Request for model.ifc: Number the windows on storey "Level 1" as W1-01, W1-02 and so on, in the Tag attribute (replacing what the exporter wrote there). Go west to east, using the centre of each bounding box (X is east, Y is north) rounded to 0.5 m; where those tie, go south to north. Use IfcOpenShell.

First a look at what the model holds.

```python
import ifcopenshell
import ifcopenshell.util.element
import ifcopenshell.util.placement

model = ifcopenshell.open("model.ifc")
print(model.schema)
storey = next(s for s in model.by_type("IfcBuildingStorey") if s.Name == "Level 1")
windows = [e for e in ifcopenshell.util.element.get_decomposition(storey) if e.is_a("IfcWindow")]
for e in sorted(windows, key=lambda e: e.id()):
    origin = ifcopenshell.util.placement.get_local_placement(e.ObjectPlacement)[:3, 3]
    print(e.id(), e.Tag, e.Name, origin.round(2) + 0.0, sep=" | ")
```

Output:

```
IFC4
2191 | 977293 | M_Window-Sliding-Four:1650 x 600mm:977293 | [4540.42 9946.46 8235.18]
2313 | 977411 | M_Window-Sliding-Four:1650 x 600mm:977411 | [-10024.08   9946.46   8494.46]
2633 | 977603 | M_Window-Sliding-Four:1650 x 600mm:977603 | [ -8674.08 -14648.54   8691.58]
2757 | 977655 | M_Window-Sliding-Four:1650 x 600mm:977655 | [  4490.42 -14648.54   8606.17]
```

```python
import ifcopenshell
import ifcopenshell.geom
import ifcopenshell.util.element
import ifcopenshell.util.shape

model = ifcopenshell.open("model.ifc")
settings = ifcopenshell.geom.settings()
settings.set("use-world-coords", True)


def centre(element):
    shape = ifcopenshell.geom.create_shape(settings, element)
    return ifcopenshell.util.shape.get_bbox_centroid(shape.geometry)


storey = next(s for s in model.by_type("IfcBuildingStorey") if s.Name == "Level 1")
windows = [e for e in ifcopenshell.util.element.get_decomposition(storey) if e.is_a("IfcWindow")]

# Insertion points can sit at a corner or the storey origin, so sort by the geometry (in metres).
centres = {e: centre(e) for e in windows}
windows.sort(key=lambda e: (round(centres[e][0] / 0.5), centres[e][1]))

for i, e in enumerate(windows, start=1):
    number = f"W1-{i:02d}"
    e.Tag = number
    print(e.id(), number)

model.write("model_edited.ifc")
```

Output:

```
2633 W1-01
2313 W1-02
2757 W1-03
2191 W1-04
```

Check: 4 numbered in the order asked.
